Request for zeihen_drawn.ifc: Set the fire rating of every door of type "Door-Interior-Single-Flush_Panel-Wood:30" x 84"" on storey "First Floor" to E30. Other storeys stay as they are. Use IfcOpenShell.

First a look at what the model holds.

```python
import ifcopenshell
import ifcopenshell.util.element

model = ifcopenshell.open("zeihen_drawn.ifc")
print(model.schema)
storey = next(s for s in model.by_type("IfcBuildingStorey") if s.Name == "First Floor")
doors = [e for e in ifcopenshell.util.element.get_decomposition(storey) if e.is_a("IfcDoor")]
seen = {}
for e in doors:
    element_type = ifcopenshell.util.element.get_type(e)
    key = (element_type.Name if element_type != e and element_type else None, ifcopenshell.util.element.get_pset(e, "Pset_DoorCommon", "FireRating"))
    seen[key] = seen.get(key, 0) + 1
for (name, value), count in sorted(seen.items(), key=str):
    print(count, "x", name, "|", value)
```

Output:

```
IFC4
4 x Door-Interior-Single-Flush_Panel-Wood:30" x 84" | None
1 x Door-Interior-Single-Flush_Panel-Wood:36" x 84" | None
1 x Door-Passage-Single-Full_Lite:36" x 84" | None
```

```python
import ifcopenshell
import ifcopenshell.api.pset
import ifcopenshell.util.element

model = ifcopenshell.open("zeihen_drawn.ifc")

storey = next(s for s in model.by_type("IfcBuildingStorey") if s.Name == "First Floor")
doors = [e for e in ifcopenshell.util.element.get_decomposition(storey) if e.is_a("IfcDoor")]

count = 0
for e in doors:
    element_type = ifcopenshell.util.element.get_type(e)
    if element_type in (None, e) or element_type.Name != 'Door-Interior-Single-Flush_Panel-Wood:30" x 84"':
        continue
    # add_pset returns the element's existing set when there is one.
    pset = ifcopenshell.api.pset.add_pset(model, product=e, name="Pset_DoorCommon")
    ifcopenshell.api.pset.edit_pset(model, pset=pset, properties={"FireRating": "E30"})
    count += 1

print(count, "doors updated")

model.write("zeihen_drawn_rev.ifc")
```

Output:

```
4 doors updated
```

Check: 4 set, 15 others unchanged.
